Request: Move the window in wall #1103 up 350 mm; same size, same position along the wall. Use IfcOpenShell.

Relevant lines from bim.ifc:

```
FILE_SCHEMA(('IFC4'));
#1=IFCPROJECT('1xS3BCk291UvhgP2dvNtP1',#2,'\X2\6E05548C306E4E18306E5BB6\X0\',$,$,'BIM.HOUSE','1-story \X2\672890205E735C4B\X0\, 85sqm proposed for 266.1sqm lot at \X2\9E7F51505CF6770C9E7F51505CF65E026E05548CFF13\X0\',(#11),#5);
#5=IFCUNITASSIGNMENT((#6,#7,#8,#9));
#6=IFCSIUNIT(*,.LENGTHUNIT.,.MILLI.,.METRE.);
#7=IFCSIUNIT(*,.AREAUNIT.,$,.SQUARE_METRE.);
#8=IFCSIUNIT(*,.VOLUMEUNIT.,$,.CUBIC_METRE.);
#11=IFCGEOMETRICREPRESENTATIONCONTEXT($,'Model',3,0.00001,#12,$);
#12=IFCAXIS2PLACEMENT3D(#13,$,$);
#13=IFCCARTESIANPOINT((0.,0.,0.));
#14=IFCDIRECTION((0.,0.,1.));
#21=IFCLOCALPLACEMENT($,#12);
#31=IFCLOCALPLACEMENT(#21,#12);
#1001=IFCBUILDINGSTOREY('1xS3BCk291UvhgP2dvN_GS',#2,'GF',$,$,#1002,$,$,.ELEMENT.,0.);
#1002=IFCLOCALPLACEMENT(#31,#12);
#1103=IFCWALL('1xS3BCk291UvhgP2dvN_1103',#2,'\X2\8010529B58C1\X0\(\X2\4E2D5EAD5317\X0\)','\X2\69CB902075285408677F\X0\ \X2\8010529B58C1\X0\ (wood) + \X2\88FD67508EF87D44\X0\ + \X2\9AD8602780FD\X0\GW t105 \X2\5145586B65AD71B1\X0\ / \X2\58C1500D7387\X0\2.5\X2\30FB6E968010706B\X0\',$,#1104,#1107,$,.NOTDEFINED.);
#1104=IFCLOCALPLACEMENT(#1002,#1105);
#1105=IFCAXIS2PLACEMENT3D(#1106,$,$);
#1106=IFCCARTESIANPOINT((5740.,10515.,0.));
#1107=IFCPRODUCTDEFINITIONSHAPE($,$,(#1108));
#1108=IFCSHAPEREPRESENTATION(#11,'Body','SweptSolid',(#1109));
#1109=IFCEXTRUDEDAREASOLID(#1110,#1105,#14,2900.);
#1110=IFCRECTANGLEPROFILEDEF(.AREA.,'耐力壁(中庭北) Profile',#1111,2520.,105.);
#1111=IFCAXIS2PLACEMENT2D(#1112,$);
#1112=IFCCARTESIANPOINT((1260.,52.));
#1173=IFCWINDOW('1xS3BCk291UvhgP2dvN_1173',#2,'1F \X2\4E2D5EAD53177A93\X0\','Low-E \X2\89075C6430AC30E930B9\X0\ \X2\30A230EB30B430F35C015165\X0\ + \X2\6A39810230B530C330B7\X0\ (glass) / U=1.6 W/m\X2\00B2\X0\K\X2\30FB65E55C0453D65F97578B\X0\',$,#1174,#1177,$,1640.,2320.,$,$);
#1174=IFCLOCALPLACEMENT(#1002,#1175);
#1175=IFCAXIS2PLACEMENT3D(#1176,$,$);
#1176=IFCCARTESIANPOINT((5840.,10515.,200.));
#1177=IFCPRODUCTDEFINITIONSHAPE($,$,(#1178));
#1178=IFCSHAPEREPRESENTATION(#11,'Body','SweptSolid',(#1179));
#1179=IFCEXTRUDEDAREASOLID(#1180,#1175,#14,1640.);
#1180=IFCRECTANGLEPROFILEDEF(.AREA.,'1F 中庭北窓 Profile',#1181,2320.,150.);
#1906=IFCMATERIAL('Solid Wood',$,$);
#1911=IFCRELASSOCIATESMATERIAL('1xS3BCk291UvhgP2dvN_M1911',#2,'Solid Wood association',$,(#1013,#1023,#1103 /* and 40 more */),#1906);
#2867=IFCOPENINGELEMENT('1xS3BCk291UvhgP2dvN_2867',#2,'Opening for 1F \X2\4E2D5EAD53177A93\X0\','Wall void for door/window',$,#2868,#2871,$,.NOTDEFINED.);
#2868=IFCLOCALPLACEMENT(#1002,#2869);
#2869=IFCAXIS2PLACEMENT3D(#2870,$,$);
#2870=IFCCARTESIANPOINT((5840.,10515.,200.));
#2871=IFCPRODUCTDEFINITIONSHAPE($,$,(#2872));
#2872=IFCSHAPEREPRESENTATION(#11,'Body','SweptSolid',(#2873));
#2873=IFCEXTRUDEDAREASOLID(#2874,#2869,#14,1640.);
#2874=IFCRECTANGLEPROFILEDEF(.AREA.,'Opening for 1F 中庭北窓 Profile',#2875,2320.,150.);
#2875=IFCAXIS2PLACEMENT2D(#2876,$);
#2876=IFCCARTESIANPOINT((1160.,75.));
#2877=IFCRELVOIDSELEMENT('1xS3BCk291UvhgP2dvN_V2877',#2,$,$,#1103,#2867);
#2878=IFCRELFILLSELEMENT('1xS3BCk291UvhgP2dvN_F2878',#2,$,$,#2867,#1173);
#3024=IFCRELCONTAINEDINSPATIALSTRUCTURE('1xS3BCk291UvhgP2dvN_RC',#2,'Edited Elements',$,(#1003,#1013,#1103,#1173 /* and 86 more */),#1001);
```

```python
import numpy as np
import ifcopenshell
import ifcopenshell.api.geometry
import ifcopenshell.util.placement
import ifcopenshell.util.unit

model = ifcopenshell.open("bim.ifc")
unit_scale = ifcopenshell.util.unit.calculate_unit_scale(model)

window = model.by_guid("1xS3BCk291UvhgP2dvN_1173")
opening = window.FillsVoids[0].RelatingOpeningElement
dz = 350.0

shift = np.array([0.0, 0.0, dz])
# The window is not placed relative to its opening, so move both.
for product in (opening, window):
    matrix = ifcopenshell.util.placement.get_local_placement(product.ObjectPlacement)
    matrix[:3, 3] += shift
    ifcopenshell.api.geometry.edit_object_placement(model, product=product, matrix=matrix, is_si=False)

print(f"moved by {dz * unit_scale:+.3f} m")

model.write("bim-out.ifc")
```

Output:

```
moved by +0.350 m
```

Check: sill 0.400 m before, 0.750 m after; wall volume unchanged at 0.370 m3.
